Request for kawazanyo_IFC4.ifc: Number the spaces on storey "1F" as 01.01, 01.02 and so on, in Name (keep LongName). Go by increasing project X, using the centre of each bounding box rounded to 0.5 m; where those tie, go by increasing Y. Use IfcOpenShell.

First a look at what the model holds.

```python
import ifcopenshell
import ifcopenshell.util.element
import ifcopenshell.util.placement

model = ifcopenshell.open("kawazanyo_IFC4.ifc")
print(model.schema)
storey = next(s for s in model.by_type("IfcBuildingStorey") if s.Name == "1F")
spaces = [e for e in ifcopenshell.util.element.get_decomposition(storey) if e.is_a("IfcSpace")]
for e in sorted(spaces, key=lambda e: e.id()):
    origin = ifcopenshell.util.placement.get_local_placement(e.ObjectPlacement)[:3, 3]
    print(e.id(), e.Name, e.LongName, origin.round(2) + 0.0, sep=" | ")
```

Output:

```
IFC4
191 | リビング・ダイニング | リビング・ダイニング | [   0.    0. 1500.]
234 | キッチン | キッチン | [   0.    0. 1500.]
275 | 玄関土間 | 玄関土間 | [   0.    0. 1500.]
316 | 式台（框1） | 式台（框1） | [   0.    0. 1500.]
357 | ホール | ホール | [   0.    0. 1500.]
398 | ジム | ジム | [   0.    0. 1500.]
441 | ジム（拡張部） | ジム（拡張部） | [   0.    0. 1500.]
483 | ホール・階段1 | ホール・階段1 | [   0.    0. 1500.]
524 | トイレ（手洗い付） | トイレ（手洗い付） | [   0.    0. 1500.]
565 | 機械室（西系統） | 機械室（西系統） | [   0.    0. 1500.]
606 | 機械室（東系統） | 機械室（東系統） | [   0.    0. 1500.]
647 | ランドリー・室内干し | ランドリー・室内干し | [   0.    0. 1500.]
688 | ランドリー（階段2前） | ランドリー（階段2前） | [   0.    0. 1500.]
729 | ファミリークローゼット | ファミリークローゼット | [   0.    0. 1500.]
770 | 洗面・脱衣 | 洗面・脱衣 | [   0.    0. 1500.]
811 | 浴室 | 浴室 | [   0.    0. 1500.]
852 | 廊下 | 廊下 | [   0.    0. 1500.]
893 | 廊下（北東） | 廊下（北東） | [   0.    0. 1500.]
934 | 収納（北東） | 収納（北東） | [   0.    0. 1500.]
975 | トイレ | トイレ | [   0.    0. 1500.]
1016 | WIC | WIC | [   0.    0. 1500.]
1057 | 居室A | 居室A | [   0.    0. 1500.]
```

```python
import ifcopenshell
import ifcopenshell.geom
import ifcopenshell.util.element
import ifcopenshell.util.shape

model = ifcopenshell.open("kawazanyo_IFC4.ifc")
settings = ifcopenshell.geom.settings()
settings.set("use-world-coords", True)


def centre(element):
    shape = ifcopenshell.geom.create_shape(settings, element)
    return ifcopenshell.util.shape.get_bbox_centroid(shape.geometry)


storey = next(s for s in model.by_type("IfcBuildingStorey") if s.Name == "1F")
spaces = [e for e in ifcopenshell.util.element.get_decomposition(storey) if e.is_a("IfcSpace")]

# Insertion points can sit at a corner or the storey origin, so sort by the geometry (in metres).
centres = {e: centre(e) for e in spaces}
spaces.sort(key=lambda e: (round(centres[e][0] / 0.5), centres[e][1]))

for i, e in enumerate(spaces, start=1):
    number = f"01.{i:02d}"
    e.Name = number
    print(e.id(), number)

model.write("kawazanyo_IFC4_rev.ifc")
```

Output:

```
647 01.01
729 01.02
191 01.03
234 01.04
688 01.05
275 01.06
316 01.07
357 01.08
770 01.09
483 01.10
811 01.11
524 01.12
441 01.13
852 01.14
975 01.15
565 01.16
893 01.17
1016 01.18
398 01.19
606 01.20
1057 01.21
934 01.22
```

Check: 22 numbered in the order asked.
